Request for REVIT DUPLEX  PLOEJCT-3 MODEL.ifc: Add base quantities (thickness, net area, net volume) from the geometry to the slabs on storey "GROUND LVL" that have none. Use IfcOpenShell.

First a look at what the model holds.

```python
import ifcopenshell
import ifcopenshell.util.element
import ifcopenshell.util.unit

model = ifcopenshell.open("REVIT DUPLEX  PLOEJCT-3 MODEL.ifc")
print(model.schema)
for unit_type in ("LENGTHUNIT", "AREAUNIT", "VOLUMEUNIT"):
    print(unit_type, ifcopenshell.util.unit.calculate_unit_scale(model, unit_type))
storey = next(s for s in model.by_type("IfcBuildingStorey") if s.Name == "GROUND LVL")
slabs = [e for e in ifcopenshell.util.element.get_decomposition(storey) if e.is_a("IfcSlab")]
for e in sorted(slabs, key=lambda e: e.id()):
    print(e.id(), e.is_a(), e.Name, list(ifcopenshell.util.element.get_psets(e, qtos_only=True)), sep=" | ")
```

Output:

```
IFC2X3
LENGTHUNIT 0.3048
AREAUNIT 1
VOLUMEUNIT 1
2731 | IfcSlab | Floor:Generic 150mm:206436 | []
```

```python
import ifcopenshell
import ifcopenshell.api.pset
import ifcopenshell.geom
import ifcopenshell.util.element
import ifcopenshell.util.shape
import ifcopenshell.util.unit

model = ifcopenshell.open("REVIT DUPLEX  PLOEJCT-3 MODEL.ifc")
unit_scale = ifcopenshell.util.unit.calculate_unit_scale(model)
area_scale = ifcopenshell.util.unit.calculate_unit_scale(model, "AREAUNIT")
volume_scale = ifcopenshell.util.unit.calculate_unit_scale(model, "VOLUMEUNIT")
settings = ifcopenshell.geom.settings()

storey = next(s for s in model.by_type("IfcBuildingStorey") if s.Name == "GROUND LVL")
slabs = [e for e in ifcopenshell.util.element.get_decomposition(storey) if e.is_a("IfcSlab")]

for e in sorted(slabs, key=lambda e: e.id()):
    if ifcopenshell.util.element.get_psets(e, qtos_only=True, should_inherit=False):
        continue
    # Geometry comes back in metres, in the element's own axes.
    shape = ifcopenshell.geom.create_shape(settings, e)
    values = {
        "Width": ifcopenshell.util.shape.get_z(shape.geometry) / unit_scale,
        "NetArea": ifcopenshell.util.shape.get_footprint_area(shape.geometry) / area_scale,
        "NetVolume": ifcopenshell.util.shape.get_volume(shape.geometry) / volume_scale,
    }
    qto = ifcopenshell.api.pset.add_qto(model, product=e, name="BaseQuantities")
    ifcopenshell.api.pset.edit_qto(model, qto=qto, properties=values)
    print(e.id(), {k: round(v, 3) for k, v in values.items()})

model.write("REVIT DUPLEX  PLOEJCT-3 MODEL-out.ifc")
```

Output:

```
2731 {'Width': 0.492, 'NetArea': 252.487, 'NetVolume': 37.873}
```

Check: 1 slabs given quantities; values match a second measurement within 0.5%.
